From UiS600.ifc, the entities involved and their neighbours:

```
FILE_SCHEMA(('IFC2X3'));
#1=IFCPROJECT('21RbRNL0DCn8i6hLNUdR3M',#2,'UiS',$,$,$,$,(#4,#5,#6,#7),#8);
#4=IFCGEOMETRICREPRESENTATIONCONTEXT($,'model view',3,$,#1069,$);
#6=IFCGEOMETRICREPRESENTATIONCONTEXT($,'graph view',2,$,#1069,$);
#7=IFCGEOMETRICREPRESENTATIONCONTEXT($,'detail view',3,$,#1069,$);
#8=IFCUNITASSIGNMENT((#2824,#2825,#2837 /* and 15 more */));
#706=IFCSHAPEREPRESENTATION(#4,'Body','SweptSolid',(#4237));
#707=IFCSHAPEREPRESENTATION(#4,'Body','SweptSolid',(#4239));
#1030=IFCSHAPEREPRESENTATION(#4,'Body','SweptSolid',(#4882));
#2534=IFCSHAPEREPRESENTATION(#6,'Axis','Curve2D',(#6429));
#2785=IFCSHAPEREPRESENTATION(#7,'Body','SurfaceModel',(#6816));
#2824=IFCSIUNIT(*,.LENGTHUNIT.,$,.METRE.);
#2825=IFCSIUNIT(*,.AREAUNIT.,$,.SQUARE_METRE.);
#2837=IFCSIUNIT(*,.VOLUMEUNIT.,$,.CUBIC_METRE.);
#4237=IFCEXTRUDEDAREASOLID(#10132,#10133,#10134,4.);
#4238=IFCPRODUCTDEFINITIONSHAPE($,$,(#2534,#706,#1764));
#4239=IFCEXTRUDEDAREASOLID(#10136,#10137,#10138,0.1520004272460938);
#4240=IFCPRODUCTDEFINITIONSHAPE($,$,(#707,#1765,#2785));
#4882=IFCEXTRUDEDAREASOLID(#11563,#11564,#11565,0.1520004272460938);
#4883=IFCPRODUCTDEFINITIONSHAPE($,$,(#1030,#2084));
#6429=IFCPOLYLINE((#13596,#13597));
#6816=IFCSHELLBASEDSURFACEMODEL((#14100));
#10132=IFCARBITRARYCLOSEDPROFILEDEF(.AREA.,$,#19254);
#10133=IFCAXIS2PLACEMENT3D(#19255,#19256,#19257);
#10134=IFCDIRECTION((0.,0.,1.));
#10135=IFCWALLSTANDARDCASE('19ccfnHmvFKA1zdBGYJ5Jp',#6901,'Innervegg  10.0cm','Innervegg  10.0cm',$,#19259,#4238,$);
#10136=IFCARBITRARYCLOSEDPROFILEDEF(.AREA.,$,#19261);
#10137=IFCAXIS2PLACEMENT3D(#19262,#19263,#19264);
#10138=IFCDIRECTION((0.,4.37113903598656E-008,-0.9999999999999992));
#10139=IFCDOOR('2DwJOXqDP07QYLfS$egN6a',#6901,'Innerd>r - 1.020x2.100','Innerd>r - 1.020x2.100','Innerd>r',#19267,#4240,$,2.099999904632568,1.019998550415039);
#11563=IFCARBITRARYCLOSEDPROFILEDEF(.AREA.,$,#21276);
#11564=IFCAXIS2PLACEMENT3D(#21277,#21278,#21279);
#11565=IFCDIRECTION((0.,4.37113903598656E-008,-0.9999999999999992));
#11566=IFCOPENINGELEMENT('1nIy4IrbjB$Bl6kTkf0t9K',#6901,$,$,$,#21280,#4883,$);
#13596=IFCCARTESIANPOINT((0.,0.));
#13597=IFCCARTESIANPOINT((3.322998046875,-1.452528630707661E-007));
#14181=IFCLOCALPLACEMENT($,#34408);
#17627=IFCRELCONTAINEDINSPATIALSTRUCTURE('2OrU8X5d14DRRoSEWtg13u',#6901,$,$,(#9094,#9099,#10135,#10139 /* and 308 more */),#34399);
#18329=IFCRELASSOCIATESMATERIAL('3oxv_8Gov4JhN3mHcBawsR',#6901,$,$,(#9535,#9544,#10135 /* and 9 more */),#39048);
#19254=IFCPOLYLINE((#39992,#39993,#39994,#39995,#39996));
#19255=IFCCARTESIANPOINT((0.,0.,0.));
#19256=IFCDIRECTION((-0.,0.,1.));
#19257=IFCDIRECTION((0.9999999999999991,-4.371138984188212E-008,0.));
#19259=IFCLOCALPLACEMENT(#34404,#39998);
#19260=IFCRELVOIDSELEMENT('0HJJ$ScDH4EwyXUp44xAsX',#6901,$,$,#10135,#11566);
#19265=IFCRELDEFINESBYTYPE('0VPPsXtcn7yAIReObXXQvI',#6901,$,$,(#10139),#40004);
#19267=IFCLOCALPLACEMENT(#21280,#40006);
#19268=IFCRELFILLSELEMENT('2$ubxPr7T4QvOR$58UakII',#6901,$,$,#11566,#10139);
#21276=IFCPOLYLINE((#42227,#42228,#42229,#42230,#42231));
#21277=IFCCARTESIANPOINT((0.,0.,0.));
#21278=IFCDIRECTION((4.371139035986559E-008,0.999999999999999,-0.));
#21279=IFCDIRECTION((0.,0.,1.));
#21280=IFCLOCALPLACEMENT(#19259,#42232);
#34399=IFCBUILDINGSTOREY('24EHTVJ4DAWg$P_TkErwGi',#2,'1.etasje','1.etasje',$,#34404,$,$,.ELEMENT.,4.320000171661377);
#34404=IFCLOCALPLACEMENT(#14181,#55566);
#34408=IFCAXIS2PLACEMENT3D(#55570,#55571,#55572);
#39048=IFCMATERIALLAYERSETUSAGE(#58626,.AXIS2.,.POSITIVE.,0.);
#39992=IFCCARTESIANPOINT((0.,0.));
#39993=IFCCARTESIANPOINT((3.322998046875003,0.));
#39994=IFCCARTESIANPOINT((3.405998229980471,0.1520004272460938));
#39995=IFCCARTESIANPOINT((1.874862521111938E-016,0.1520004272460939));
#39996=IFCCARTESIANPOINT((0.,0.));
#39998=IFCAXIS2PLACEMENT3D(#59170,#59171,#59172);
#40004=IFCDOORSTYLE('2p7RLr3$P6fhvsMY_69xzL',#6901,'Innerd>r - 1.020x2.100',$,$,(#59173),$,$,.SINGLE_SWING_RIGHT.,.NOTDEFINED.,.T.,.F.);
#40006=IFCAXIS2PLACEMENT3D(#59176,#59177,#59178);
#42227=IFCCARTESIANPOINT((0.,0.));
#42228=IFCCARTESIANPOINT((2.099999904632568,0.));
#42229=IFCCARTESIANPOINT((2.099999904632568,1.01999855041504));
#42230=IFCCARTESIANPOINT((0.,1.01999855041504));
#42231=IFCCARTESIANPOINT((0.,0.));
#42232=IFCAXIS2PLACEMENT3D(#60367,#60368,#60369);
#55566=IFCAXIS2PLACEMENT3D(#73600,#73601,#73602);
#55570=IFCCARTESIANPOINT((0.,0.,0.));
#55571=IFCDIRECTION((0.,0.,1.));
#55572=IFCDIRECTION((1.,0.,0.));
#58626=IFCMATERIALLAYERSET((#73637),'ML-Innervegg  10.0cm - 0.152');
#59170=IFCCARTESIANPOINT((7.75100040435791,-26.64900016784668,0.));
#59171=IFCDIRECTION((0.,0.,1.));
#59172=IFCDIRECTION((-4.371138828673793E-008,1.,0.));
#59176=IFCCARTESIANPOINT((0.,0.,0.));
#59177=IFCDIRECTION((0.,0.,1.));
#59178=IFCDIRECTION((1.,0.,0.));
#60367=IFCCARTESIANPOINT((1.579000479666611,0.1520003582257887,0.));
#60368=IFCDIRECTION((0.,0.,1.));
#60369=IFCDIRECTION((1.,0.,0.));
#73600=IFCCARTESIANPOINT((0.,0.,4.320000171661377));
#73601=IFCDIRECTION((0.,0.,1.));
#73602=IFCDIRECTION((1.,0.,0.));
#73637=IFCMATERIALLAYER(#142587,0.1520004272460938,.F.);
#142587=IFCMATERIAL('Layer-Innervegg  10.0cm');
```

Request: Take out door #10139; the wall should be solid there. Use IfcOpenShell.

```python
import ifcopenshell
import ifcopenshell.api.feature
import ifcopenshell.api.root
import ifcopenshell.geom
import ifcopenshell.util.shape

model = ifcopenshell.open("UiS600.ifc")
settings = ifcopenshell.geom.settings()


def volume(element):
    """Net volume in cubic metres, openings subtracted."""
    shape = ifcopenshell.geom.create_shape(settings, element)
    return ifcopenshell.util.shape.get_volume(shape.geometry)


door = model.by_id(10139)
opening = door.FillsVoids[0].RelatingOpeningElement
wall = opening.VoidsElements[0].RelatingBuildingElement
before = volume(wall)

ifcopenshell.api.root.remove_product(model, product=door)
ifcopenshell.api.feature.remove_feature(model, feature=opening)

after = volume(wall)

print(f"wall volume {before:.3f} -> {after:.3f} m3")

model.write("UiS600_updated.ifc")
```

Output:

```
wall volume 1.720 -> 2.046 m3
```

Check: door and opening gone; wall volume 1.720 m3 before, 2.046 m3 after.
